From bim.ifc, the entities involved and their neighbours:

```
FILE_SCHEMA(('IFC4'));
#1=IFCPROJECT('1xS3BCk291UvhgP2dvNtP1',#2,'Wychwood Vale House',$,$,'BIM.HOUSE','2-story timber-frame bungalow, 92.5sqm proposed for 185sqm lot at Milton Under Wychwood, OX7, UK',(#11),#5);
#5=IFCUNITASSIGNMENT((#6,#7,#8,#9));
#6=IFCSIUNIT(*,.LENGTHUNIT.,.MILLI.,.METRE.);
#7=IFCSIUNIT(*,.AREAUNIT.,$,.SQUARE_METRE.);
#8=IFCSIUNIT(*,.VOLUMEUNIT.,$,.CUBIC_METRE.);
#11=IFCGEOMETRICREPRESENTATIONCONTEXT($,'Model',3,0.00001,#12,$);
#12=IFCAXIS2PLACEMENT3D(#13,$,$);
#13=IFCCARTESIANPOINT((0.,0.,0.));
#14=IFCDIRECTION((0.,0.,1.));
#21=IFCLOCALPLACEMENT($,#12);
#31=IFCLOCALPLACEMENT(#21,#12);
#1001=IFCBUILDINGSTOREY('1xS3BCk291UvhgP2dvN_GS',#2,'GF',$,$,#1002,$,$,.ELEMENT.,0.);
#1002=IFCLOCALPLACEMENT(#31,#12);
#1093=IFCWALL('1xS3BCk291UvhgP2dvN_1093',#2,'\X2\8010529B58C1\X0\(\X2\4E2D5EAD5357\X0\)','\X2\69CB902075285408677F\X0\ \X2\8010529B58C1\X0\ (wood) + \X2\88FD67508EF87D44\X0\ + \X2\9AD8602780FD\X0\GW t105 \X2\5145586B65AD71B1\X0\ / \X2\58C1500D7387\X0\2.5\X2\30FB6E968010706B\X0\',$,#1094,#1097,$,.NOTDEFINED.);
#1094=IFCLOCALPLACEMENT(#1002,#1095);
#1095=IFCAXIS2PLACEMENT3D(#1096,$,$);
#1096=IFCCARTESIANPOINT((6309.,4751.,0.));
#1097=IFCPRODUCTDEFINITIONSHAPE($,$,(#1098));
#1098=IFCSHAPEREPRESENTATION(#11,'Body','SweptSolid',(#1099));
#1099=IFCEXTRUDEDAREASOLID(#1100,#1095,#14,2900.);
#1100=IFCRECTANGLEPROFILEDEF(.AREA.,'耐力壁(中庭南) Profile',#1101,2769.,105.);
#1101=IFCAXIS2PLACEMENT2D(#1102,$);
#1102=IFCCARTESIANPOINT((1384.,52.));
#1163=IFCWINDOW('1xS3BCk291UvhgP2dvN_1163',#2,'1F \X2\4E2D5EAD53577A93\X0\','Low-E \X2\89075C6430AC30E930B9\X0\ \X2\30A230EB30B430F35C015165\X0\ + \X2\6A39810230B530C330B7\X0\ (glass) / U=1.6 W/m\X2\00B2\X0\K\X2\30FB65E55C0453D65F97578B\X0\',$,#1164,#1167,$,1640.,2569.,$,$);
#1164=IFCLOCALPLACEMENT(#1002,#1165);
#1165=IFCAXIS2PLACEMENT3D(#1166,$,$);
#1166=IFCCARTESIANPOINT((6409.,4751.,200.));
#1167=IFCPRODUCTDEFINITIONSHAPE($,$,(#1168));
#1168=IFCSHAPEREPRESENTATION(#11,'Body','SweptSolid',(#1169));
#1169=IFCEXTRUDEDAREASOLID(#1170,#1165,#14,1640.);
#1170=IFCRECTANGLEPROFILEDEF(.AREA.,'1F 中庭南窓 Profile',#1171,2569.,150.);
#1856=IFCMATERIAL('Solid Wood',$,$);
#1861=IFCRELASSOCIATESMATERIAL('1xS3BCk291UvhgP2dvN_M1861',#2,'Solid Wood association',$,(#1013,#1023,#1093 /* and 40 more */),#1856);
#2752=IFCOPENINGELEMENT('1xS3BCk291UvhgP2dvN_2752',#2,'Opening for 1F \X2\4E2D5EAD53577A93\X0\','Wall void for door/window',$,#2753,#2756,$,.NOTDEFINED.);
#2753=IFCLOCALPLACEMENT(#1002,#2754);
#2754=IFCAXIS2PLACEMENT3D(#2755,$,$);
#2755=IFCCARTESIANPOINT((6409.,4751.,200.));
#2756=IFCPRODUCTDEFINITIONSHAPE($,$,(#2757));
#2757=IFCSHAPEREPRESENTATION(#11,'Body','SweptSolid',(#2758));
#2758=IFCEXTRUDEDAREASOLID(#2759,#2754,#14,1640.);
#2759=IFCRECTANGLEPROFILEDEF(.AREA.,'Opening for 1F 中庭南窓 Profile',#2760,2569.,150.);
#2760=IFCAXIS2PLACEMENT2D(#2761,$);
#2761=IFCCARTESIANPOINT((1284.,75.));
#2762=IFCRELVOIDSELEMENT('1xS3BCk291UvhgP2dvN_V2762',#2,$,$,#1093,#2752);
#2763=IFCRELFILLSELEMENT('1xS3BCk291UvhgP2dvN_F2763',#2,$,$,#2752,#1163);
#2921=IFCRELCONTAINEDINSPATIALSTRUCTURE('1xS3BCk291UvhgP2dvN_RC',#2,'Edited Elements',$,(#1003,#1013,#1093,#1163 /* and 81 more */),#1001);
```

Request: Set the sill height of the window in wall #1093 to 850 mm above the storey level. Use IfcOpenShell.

```python
import numpy as np
import ifcopenshell
import ifcopenshell.api.geometry
import ifcopenshell.geom
import ifcopenshell.util.element
import ifcopenshell.util.placement
import ifcopenshell.util.shape
import ifcopenshell.util.unit

model = ifcopenshell.open("bim.ifc")
unit_scale = ifcopenshell.util.unit.calculate_unit_scale(model)

window = model.by_guid("1xS3BCk291UvhgP2dvN_1163")
opening = window.FillsVoids[0].RelatingOpeningElement
storey = ifcopenshell.util.element.get_container(window, ifc_class="IfcBuildingStorey")
level = ifcopenshell.util.placement.get_local_placement(storey.ObjectPlacement)[2, 3]

# The opening's origin need not be at the sill, so measure its lowest point.
shape = ifcopenshell.geom.create_shape(ifcopenshell.geom.settings(), opening)
bottom = ifcopenshell.util.shape.get_shape_bottom_elevation(shape, shape.geometry) / unit_scale
dz = level + 850.0 - bottom

shift = np.array([0.0, 0.0, dz])
# The window is not placed relative to its opening, so move both.
for product in (opening, window):
    matrix = ifcopenshell.util.placement.get_local_placement(product.ObjectPlacement)
    matrix[:3, 3] += shift
    ifcopenshell.api.geometry.edit_object_placement(model, product=product, matrix=matrix, is_si=False)

print(f"moved by {dz * unit_scale:+.3f} m")

model.write("bim_edited.ifc")
```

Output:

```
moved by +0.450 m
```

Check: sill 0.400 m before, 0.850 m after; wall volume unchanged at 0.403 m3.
